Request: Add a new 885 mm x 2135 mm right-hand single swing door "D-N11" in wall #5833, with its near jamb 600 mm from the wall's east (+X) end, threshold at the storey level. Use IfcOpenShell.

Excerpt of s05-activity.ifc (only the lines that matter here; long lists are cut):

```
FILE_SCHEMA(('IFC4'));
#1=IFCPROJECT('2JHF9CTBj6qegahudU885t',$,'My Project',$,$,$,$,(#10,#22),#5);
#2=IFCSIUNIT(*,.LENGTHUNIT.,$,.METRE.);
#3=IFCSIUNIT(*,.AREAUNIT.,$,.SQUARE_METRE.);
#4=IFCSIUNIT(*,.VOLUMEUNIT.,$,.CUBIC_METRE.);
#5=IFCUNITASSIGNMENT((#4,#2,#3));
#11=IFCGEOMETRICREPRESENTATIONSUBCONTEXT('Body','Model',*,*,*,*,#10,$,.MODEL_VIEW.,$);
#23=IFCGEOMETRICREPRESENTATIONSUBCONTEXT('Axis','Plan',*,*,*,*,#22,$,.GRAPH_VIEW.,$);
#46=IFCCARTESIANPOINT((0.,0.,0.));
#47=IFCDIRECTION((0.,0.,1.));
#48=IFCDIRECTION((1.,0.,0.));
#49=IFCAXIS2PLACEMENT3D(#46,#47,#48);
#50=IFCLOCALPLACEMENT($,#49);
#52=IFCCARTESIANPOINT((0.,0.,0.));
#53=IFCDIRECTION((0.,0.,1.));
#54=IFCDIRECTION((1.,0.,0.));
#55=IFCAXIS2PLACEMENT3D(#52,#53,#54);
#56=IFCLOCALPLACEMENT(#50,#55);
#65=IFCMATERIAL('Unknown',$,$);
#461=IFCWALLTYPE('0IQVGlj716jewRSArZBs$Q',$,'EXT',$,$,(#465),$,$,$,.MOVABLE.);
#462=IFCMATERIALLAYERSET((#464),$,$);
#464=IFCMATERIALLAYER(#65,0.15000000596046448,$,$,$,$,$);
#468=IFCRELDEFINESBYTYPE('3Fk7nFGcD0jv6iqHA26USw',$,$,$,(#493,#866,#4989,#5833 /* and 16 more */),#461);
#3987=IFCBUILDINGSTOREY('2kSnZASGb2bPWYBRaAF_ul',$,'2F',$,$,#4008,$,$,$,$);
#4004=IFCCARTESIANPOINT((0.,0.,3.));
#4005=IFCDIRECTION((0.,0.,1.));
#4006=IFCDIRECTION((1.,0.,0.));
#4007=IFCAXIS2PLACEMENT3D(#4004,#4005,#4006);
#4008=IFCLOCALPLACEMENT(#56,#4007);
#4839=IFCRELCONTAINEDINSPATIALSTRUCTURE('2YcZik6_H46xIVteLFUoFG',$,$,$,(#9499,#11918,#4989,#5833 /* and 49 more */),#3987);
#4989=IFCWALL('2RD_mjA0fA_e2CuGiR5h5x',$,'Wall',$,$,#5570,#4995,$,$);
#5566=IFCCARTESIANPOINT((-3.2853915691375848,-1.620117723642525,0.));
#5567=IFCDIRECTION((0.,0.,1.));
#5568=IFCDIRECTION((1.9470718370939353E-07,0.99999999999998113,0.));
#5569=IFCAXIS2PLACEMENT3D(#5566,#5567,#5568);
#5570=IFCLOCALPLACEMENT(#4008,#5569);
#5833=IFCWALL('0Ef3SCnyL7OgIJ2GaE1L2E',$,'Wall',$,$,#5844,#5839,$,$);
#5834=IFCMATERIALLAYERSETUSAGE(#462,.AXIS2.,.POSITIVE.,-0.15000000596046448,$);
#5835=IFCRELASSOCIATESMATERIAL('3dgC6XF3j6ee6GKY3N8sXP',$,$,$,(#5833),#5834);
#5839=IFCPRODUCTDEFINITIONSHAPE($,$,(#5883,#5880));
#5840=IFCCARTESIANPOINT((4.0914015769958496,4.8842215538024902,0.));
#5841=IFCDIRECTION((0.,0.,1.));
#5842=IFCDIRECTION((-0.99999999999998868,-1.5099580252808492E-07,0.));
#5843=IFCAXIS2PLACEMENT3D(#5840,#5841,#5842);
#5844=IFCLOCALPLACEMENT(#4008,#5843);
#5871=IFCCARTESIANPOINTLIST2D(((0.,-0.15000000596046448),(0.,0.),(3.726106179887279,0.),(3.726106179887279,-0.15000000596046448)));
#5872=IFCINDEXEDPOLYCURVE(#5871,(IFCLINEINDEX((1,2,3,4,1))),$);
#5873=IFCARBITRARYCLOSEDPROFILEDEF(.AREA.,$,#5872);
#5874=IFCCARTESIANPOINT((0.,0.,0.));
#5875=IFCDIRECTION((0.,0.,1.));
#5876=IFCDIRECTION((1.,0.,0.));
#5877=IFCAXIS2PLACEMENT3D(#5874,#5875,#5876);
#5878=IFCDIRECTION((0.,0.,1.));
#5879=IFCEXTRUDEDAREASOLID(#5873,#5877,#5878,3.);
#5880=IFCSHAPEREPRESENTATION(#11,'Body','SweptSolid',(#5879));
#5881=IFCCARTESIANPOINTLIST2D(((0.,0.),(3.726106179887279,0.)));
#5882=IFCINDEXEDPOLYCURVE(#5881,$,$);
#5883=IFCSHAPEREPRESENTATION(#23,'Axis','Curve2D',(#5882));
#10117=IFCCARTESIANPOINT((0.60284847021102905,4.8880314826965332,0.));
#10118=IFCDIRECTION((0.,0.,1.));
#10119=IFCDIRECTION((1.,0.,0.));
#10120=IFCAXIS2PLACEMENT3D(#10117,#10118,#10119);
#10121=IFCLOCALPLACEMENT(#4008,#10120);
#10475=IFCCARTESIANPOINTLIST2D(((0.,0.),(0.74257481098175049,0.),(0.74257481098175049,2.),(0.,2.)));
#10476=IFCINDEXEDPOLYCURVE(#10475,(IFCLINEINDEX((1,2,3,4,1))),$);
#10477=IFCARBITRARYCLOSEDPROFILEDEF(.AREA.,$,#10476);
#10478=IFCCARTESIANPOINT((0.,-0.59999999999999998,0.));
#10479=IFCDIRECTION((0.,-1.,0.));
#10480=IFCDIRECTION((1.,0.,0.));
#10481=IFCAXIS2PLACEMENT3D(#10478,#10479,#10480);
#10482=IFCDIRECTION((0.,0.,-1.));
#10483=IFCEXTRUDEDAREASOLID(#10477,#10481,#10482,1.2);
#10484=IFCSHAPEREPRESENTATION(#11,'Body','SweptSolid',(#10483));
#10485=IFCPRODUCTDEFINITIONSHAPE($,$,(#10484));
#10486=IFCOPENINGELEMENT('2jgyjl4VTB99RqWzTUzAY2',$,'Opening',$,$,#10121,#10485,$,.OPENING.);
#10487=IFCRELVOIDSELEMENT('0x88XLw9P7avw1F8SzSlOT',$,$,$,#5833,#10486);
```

```python
import numpy as np
import ifcopenshell
import ifcopenshell.api.feature
import ifcopenshell.api.geometry
import ifcopenshell.api.root
import ifcopenshell.api.spatial
import ifcopenshell.geom
import ifcopenshell.util.element
import ifcopenshell.util.placement
import ifcopenshell.util.representation
import ifcopenshell.util.shape
import ifcopenshell.util.unit

model = ifcopenshell.open("s05-activity.ifc")
unit_scale = ifcopenshell.util.unit.calculate_unit_scale(model)
settings = ifcopenshell.geom.settings()


def volume(element):
    """Net volume in cubic metres, openings subtracted."""
    shape = ifcopenshell.geom.create_shape(settings, element)
    return ifcopenshell.util.shape.get_volume(shape.geometry)


wall = model.by_guid("0Ef3SCnyL7OgIJ2GaE1L2E")
storey = ifcopenshell.util.element.get_container(wall, ifc_class="IfcBuildingStorey")
context = ifcopenshell.util.representation.get_context(model, "Model", "Body", "MODEL_VIEW")
before = volume(wall)

width, height, from_end, sill = 0.885, 2.135, 0.6, 0.0  # metres

# The wall runs along its own X axis, and the end named is its -X end.
wall_shape = ifcopenshell.geom.create_shape(settings, wall)
x, y, z = ifcopenshell.util.shape.get_vertices(wall_shape.geometry).T
start = x.min() + from_end
face, thickness = float(y.min()), float(y.max() - y.min())
wall_matrix = ifcopenshell.util.placement.get_local_placement(wall.ObjectPlacement)
level = ifcopenshell.util.placement.get_local_placement(storey.ObjectPlacement)[2, 3]


def in_wall(x, y):
    """Placement at x, y metres in the wall's axes, at sill height."""
    matrix = wall_matrix.copy()
    matrix[:, 3] = wall_matrix @ np.array([x / unit_scale, y / unit_scale, 0.0, 1.0])
    matrix[2, 3] = level + sill / unit_scale
    return matrix


# Opening: a box that overshoots both wall faces by 50 mm.
opening = ifcopenshell.api.root.create_entity(model, ifc_class="IfcOpeningElement", predefined_type="OPENING")
box = ifcopenshell.api.geometry.add_wall_representation(
    model, context=context, length=width, height=height, thickness=thickness + 0.1
)
ifcopenshell.api.geometry.assign_representation(model, product=opening, representation=box)
ifcopenshell.api.geometry.edit_object_placement(model, product=opening, matrix=in_wall(start, face - 0.05), is_si=False)
ifcopenshell.api.feature.add_feature(model, feature=opening, element=wall)

door = ifcopenshell.api.root.create_entity(model, ifc_class="IfcDoor", name="D-N11", predefined_type="DOOR")
door.OverallWidth, door.OverallHeight = width / unit_scale, height / unit_scale
door.OperationType = "SINGLE_SWING_RIGHT"
body = ifcopenshell.api.geometry.add_door_representation(
    model,
    context=context,
    overall_width=door.OverallWidth,
    overall_height=door.OverallHeight,
    operation_type="SINGLE_SWING_RIGHT",
    lining_properties={"LiningDepth": thickness / unit_scale, "ThresholdDepth": thickness / unit_scale},
)
ifcopenshell.api.geometry.assign_representation(model, product=door, representation=body)
ifcopenshell.api.spatial.assign_container(model, products=[door], relating_structure=storey)
ifcopenshell.api.feature.add_filling(model, opening=opening, element=door)

# The lining spans the wall, so the door starts at the wall face.
ifcopenshell.api.geometry.edit_object_placement(model, product=door, matrix=in_wall(start, face), is_si=False)

after = volume(wall)

print(f"wall volume {before:.3f} -> {after:.3f} m3")

model.write("s05-activity_v2.ifc")
```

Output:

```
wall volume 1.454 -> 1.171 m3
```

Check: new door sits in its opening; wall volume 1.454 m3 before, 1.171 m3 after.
